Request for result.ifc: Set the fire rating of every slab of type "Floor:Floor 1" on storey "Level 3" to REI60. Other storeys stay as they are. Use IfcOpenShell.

First a look at what the model holds.

```python
import ifcopenshell
import ifcopenshell.util.element

model = ifcopenshell.open("result.ifc")
print(model.schema)
storey = next(s for s in model.by_type("IfcBuildingStorey") if s.Name == "Level 3")
slabs = [e for e in ifcopenshell.util.element.get_decomposition(storey) if e.is_a("IfcSlab")]
seen = {}
for e in slabs:
    element_type = ifcopenshell.util.element.get_type(e)
    key = (element_type.Name if element_type != e and element_type else None, ifcopenshell.util.element.get_pset(e, "Pset_SlabCommon", "FireRating"))
    seen[key] = seen.get(key, 0) + 1
for (name, value), count in sorted(seen.items(), key=str):
    print(count, "x", name, "|", value)
```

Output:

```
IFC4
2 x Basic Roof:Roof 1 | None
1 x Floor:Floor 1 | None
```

```python
import ifcopenshell
import ifcopenshell.api.pset
import ifcopenshell.util.element

model = ifcopenshell.open("result.ifc")

storey = next(s for s in model.by_type("IfcBuildingStorey") if s.Name == "Level 3")
slabs = [e for e in ifcopenshell.util.element.get_decomposition(storey) if e.is_a("IfcSlab")]

count = 0
for e in slabs:
    element_type = ifcopenshell.util.element.get_type(e)
    if element_type in (None, e) or element_type.Name != "Floor:Floor 1":
        continue
    # add_pset returns the element's existing set when there is one.
    pset = ifcopenshell.api.pset.add_pset(model, product=e, name="Pset_SlabCommon")
    ifcopenshell.api.pset.edit_pset(model, pset=pset, properties={"FireRating": "REI60"})
    count += 1

print(count, "slabs updated")

model.write("result_updated.ifc")
```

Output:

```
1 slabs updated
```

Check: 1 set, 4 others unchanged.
